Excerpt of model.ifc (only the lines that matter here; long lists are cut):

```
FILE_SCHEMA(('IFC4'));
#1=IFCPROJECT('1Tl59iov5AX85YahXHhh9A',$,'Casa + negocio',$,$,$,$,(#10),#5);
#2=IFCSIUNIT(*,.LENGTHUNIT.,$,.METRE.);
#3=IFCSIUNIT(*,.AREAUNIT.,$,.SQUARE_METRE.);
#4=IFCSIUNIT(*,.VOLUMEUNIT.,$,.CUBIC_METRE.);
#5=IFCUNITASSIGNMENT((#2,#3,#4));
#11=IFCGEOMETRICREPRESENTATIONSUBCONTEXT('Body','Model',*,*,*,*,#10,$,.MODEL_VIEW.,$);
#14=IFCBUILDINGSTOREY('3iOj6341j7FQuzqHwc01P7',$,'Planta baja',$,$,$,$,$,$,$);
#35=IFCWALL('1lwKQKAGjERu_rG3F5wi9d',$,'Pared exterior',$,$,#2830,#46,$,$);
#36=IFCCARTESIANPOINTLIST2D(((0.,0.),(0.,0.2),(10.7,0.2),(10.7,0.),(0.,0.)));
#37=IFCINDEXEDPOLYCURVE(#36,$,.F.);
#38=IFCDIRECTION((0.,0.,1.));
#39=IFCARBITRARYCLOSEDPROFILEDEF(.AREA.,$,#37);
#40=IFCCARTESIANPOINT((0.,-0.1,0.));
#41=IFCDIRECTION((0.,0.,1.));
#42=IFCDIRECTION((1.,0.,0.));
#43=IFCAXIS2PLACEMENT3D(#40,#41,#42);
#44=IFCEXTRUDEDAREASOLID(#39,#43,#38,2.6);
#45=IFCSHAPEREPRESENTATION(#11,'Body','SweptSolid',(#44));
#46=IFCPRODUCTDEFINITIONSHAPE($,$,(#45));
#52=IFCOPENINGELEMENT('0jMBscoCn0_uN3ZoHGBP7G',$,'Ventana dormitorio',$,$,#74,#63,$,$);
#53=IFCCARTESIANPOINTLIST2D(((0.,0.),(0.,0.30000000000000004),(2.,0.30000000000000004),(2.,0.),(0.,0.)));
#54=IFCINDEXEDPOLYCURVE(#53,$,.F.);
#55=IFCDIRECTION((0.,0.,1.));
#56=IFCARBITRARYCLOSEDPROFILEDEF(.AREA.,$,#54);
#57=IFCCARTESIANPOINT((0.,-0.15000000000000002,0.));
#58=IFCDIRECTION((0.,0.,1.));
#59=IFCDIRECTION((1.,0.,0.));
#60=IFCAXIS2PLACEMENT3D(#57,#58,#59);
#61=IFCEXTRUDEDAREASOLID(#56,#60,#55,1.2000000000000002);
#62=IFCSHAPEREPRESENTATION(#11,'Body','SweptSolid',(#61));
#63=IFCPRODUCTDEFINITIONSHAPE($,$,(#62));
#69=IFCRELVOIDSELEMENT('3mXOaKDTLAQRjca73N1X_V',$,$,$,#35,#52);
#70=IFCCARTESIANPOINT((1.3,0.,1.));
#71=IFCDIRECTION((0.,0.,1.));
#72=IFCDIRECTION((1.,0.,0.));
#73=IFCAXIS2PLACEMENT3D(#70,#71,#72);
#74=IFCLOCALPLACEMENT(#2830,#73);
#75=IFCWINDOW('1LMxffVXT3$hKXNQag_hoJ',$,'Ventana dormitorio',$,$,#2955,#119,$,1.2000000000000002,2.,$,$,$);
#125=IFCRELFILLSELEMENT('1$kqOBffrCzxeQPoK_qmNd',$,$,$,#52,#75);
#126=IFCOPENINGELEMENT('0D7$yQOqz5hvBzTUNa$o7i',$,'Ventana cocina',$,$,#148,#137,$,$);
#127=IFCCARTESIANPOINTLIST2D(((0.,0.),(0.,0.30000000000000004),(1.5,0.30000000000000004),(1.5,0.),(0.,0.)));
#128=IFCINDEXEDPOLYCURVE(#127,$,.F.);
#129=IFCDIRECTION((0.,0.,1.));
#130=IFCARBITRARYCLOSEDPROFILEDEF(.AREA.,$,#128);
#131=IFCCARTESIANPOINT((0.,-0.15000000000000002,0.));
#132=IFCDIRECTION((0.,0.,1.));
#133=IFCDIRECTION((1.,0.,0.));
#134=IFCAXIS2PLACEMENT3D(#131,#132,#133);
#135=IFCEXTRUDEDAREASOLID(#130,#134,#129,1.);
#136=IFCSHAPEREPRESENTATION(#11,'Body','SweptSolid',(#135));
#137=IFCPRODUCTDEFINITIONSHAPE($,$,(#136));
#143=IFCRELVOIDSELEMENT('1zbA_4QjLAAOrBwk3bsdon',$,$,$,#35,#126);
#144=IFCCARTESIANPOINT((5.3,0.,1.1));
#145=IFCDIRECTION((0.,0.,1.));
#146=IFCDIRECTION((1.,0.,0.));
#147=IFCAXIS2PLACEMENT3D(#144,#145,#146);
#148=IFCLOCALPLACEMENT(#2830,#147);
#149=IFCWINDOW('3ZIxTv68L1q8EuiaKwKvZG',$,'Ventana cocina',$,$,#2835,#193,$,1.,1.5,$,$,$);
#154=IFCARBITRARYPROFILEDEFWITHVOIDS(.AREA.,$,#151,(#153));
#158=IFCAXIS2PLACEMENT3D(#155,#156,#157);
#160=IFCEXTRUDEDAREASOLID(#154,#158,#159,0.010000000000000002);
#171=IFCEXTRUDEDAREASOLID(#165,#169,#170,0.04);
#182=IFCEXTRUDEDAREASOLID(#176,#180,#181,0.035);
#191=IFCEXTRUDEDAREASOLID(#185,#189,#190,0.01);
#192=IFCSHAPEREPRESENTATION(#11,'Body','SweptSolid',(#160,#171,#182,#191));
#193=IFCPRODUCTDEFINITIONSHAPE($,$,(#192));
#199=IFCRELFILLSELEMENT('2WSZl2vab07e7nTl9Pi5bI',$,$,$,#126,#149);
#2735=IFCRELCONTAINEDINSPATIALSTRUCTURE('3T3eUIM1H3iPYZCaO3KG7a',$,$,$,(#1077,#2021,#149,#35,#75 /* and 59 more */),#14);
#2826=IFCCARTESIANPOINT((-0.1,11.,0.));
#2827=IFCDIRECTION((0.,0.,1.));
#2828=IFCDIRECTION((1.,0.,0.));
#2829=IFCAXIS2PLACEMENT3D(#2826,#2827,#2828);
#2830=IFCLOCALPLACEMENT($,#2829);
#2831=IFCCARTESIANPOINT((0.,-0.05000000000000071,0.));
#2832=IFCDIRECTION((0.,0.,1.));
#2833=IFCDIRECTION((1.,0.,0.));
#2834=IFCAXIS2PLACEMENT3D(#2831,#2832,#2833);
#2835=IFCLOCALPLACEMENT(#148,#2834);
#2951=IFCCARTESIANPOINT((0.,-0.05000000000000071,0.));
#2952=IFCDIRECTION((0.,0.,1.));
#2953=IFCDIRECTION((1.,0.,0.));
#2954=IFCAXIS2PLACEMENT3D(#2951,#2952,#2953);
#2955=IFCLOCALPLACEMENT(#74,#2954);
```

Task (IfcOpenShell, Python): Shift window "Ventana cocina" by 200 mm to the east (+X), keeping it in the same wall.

```python
import ifcopenshell
import ifcopenshell.api.geometry
import ifcopenshell.util.placement

model = ifcopenshell.open("model.ifc")

window = model.by_guid("3ZIxTv68L1q8EuiaKwKvZG")
opening = window.FillsVoids[0].RelatingOpeningElement
wall = opening.VoidsElements[0].RelatingBuildingElement

wall_matrix = ifcopenshell.util.placement.get_local_placement(wall.ObjectPlacement)
shift = wall_matrix[:3, 0] * 0.2
before = ifcopenshell.util.placement.get_local_placement(window.ObjectPlacement)[:3, 3].copy()

# The window is placed relative to its opening, so it follows when the opening moves.
matrix = ifcopenshell.util.placement.get_local_placement(opening.ObjectPlacement)
matrix[:3, 3] += shift
ifcopenshell.api.geometry.edit_object_placement(
    model, product=opening, matrix=matrix, is_si=False, should_transform_children=True
)

after = ifcopenshell.util.placement.get_local_placement(window.ObjectPlacement)[:3, 3]
print("window moved by", (after - before).round(3) + 0.0)

model.write("model_updated.ifc")
```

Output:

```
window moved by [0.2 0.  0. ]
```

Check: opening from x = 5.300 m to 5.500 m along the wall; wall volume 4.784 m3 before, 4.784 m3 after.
